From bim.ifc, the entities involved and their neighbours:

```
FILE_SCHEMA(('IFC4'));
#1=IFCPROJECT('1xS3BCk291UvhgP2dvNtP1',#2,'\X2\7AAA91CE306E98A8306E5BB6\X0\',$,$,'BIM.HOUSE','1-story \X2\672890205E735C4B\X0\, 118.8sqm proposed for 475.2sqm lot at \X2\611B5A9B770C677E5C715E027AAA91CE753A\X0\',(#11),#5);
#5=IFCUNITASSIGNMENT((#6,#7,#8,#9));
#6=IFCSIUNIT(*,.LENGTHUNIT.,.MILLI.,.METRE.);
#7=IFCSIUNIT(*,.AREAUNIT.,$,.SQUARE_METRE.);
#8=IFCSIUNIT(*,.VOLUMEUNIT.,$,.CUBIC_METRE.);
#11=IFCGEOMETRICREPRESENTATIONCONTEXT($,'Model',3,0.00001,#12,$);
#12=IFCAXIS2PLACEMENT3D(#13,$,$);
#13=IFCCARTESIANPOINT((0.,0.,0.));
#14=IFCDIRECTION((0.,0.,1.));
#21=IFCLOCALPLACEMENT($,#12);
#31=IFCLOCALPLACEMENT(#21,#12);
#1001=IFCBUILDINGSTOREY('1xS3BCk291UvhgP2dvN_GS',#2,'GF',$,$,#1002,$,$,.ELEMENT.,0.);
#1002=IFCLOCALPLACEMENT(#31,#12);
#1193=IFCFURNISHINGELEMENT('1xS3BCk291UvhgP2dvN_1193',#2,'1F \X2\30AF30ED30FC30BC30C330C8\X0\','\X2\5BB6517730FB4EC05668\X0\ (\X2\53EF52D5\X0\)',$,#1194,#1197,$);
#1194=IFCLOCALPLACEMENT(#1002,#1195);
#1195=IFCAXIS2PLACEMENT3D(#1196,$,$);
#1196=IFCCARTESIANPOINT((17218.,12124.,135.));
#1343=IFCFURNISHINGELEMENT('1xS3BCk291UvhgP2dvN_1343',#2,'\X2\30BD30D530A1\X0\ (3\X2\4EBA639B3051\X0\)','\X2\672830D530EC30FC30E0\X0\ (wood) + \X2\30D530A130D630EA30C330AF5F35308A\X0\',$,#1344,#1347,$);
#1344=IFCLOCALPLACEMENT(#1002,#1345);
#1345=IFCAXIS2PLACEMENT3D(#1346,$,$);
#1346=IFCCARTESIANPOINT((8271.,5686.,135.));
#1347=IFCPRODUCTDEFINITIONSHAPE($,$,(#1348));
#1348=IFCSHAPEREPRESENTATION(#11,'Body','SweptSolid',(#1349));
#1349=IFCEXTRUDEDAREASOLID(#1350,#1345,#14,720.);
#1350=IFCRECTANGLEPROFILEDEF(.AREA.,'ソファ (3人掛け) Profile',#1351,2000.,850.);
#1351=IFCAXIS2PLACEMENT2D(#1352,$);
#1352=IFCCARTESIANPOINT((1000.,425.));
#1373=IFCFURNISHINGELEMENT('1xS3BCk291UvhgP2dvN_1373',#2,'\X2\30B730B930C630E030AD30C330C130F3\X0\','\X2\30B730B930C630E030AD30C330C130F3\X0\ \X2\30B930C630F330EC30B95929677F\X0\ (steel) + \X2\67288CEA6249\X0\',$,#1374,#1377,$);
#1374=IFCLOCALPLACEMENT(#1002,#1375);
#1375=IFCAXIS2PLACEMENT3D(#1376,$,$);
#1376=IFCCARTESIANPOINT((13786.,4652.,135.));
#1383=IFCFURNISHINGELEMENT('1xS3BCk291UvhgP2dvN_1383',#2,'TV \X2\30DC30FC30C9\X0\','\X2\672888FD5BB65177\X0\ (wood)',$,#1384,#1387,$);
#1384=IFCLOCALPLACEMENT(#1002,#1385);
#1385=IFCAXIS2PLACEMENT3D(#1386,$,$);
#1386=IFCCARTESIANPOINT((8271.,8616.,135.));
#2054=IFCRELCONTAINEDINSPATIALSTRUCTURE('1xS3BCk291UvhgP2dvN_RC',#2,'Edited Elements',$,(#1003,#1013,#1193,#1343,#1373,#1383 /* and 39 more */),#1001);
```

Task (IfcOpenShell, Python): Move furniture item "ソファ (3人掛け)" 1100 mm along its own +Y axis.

```python
import ifcopenshell
import ifcopenshell.api.geometry
import ifcopenshell.util.placement
import ifcopenshell.util.unit

model = ifcopenshell.open("bim.ifc")
unit_scale = ifcopenshell.util.unit.calculate_unit_scale(model)

item = model.by_guid("1xS3BCk291UvhgP2dvN_1343")
matrix = ifcopenshell.util.placement.get_local_placement(item.ObjectPlacement)
matrix[:3, 3] += matrix[:3, 1] * 1.1 / unit_scale
ifcopenshell.api.geometry.edit_object_placement(model, product=item, matrix=matrix, is_si=False)

print(ifcopenshell.util.placement.get_local_placement(item.ObjectPlacement).round(3) + 0.0)

model.write("bim_v2.ifc")
```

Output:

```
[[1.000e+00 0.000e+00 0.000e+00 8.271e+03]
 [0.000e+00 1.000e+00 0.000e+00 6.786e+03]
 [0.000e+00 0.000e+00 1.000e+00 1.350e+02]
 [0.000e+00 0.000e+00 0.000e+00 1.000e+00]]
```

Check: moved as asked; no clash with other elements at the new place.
